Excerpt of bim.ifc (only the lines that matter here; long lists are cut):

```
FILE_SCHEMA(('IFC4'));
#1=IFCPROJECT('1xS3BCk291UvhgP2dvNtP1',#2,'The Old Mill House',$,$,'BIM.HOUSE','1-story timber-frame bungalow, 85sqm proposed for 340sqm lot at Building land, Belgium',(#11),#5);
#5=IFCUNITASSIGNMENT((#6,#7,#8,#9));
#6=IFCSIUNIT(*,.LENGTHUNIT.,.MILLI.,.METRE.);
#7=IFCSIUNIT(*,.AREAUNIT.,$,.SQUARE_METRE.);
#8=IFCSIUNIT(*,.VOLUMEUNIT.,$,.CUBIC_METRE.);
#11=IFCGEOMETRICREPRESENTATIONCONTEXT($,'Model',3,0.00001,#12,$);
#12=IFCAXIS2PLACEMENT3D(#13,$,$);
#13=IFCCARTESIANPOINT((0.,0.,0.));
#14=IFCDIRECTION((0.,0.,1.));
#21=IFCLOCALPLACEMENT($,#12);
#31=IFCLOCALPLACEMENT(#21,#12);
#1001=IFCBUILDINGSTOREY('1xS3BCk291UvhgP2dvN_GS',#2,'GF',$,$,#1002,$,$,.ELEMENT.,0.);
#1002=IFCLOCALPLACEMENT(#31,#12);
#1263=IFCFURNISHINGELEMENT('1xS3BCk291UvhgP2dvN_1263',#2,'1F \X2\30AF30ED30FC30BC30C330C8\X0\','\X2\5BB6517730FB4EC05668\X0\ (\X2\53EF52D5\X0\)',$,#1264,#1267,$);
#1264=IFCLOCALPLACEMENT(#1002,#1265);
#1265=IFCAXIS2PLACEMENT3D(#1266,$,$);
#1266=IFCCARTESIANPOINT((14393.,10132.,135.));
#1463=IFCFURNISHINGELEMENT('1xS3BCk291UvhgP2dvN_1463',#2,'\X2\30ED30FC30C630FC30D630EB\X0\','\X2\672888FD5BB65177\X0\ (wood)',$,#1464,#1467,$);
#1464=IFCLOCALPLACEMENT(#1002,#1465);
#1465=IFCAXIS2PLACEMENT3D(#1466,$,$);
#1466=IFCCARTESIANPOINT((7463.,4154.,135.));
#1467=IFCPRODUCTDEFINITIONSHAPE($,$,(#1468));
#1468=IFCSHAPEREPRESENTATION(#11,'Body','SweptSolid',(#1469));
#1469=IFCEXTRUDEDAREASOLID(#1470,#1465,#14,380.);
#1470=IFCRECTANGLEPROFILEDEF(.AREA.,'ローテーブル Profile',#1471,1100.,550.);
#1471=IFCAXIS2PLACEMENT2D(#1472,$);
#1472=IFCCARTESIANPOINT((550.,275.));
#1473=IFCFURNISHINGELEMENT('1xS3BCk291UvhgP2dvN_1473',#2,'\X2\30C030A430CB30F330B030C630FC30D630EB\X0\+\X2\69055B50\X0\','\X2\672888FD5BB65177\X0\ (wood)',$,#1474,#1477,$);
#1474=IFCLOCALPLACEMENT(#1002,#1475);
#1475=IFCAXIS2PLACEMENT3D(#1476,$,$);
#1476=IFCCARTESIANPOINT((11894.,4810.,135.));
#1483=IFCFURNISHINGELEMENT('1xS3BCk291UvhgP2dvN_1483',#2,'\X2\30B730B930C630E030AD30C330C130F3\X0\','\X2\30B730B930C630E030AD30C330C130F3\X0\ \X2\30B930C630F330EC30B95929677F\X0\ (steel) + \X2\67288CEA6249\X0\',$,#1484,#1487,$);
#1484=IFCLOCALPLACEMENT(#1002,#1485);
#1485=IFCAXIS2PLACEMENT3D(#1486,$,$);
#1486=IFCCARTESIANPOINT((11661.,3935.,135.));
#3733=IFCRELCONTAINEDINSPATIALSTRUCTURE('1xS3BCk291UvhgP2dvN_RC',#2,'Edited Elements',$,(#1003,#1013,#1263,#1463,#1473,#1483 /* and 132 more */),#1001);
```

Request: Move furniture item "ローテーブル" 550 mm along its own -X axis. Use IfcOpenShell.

```python
import ifcopenshell
import ifcopenshell.api.geometry
import ifcopenshell.util.placement
import ifcopenshell.util.unit

model = ifcopenshell.open("bim.ifc")
unit_scale = ifcopenshell.util.unit.calculate_unit_scale(model)

item = model.by_guid("1xS3BCk291UvhgP2dvN_1463")
matrix = ifcopenshell.util.placement.get_local_placement(item.ObjectPlacement)
matrix[:3, 3] -= matrix[:3, 0] * 0.55 / unit_scale
ifcopenshell.api.geometry.edit_object_placement(model, product=item, matrix=matrix, is_si=False)

print(ifcopenshell.util.placement.get_local_placement(item.ObjectPlacement).round(3) + 0.0)

model.write("bim_v2.ifc")
```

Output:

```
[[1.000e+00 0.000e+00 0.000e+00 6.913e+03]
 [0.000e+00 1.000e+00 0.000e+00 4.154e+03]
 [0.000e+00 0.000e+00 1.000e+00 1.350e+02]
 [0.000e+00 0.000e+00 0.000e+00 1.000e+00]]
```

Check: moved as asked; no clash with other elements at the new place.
